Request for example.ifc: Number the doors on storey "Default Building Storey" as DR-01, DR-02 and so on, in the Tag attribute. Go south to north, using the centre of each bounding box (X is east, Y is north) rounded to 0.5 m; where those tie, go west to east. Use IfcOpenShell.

First a look at what the model holds.

```python
import ifcopenshell
import ifcopenshell.util.element
import ifcopenshell.util.placement

model = ifcopenshell.open("example.ifc")
print(model.schema)
storey = next(s for s in model.by_type("IfcBuildingStorey") if s.Name == "Default Building Storey")
doors = [e for e in ifcopenshell.util.element.get_decomposition(storey) if e.is_a("IfcDoor")]
for e in sorted(doors, key=lambda e: e.id()):
    origin = ifcopenshell.util.placement.get_local_placement(e.ObjectPlacement)[:3, 3]
    print(e.id(), e.Tag, e.Name, origin.round(2) + 0.0, sep=" | ")
```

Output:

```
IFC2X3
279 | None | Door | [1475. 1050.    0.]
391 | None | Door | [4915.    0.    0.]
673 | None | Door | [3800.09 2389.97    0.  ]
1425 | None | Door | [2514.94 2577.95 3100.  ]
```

```python
import ifcopenshell
import ifcopenshell.geom
import ifcopenshell.util.element
import ifcopenshell.util.shape

model = ifcopenshell.open("example.ifc")
settings = ifcopenshell.geom.settings()
settings.set("use-world-coords", True)


def centre(element):
    shape = ifcopenshell.geom.create_shape(settings, element)
    return ifcopenshell.util.shape.get_bbox_centroid(shape.geometry)


storey = next(s for s in model.by_type("IfcBuildingStorey") if s.Name == "Default Building Storey")
doors = [e for e in ifcopenshell.util.element.get_decomposition(storey) if e.is_a("IfcDoor")]

# Insertion points can sit at a corner or the storey origin, so sort by the geometry (in metres).
centres = {e: centre(e) for e in doors}
doors.sort(key=lambda e: (round(centres[e][1] / 0.5), centres[e][0]))

for i, e in enumerate(doors, start=1):
    number = f"DR-{i:02d}"
    e.Tag = number
    print(e.id(), number)

model.write("example-out.ifc")
```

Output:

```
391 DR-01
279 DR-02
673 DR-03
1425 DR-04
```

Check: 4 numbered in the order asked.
